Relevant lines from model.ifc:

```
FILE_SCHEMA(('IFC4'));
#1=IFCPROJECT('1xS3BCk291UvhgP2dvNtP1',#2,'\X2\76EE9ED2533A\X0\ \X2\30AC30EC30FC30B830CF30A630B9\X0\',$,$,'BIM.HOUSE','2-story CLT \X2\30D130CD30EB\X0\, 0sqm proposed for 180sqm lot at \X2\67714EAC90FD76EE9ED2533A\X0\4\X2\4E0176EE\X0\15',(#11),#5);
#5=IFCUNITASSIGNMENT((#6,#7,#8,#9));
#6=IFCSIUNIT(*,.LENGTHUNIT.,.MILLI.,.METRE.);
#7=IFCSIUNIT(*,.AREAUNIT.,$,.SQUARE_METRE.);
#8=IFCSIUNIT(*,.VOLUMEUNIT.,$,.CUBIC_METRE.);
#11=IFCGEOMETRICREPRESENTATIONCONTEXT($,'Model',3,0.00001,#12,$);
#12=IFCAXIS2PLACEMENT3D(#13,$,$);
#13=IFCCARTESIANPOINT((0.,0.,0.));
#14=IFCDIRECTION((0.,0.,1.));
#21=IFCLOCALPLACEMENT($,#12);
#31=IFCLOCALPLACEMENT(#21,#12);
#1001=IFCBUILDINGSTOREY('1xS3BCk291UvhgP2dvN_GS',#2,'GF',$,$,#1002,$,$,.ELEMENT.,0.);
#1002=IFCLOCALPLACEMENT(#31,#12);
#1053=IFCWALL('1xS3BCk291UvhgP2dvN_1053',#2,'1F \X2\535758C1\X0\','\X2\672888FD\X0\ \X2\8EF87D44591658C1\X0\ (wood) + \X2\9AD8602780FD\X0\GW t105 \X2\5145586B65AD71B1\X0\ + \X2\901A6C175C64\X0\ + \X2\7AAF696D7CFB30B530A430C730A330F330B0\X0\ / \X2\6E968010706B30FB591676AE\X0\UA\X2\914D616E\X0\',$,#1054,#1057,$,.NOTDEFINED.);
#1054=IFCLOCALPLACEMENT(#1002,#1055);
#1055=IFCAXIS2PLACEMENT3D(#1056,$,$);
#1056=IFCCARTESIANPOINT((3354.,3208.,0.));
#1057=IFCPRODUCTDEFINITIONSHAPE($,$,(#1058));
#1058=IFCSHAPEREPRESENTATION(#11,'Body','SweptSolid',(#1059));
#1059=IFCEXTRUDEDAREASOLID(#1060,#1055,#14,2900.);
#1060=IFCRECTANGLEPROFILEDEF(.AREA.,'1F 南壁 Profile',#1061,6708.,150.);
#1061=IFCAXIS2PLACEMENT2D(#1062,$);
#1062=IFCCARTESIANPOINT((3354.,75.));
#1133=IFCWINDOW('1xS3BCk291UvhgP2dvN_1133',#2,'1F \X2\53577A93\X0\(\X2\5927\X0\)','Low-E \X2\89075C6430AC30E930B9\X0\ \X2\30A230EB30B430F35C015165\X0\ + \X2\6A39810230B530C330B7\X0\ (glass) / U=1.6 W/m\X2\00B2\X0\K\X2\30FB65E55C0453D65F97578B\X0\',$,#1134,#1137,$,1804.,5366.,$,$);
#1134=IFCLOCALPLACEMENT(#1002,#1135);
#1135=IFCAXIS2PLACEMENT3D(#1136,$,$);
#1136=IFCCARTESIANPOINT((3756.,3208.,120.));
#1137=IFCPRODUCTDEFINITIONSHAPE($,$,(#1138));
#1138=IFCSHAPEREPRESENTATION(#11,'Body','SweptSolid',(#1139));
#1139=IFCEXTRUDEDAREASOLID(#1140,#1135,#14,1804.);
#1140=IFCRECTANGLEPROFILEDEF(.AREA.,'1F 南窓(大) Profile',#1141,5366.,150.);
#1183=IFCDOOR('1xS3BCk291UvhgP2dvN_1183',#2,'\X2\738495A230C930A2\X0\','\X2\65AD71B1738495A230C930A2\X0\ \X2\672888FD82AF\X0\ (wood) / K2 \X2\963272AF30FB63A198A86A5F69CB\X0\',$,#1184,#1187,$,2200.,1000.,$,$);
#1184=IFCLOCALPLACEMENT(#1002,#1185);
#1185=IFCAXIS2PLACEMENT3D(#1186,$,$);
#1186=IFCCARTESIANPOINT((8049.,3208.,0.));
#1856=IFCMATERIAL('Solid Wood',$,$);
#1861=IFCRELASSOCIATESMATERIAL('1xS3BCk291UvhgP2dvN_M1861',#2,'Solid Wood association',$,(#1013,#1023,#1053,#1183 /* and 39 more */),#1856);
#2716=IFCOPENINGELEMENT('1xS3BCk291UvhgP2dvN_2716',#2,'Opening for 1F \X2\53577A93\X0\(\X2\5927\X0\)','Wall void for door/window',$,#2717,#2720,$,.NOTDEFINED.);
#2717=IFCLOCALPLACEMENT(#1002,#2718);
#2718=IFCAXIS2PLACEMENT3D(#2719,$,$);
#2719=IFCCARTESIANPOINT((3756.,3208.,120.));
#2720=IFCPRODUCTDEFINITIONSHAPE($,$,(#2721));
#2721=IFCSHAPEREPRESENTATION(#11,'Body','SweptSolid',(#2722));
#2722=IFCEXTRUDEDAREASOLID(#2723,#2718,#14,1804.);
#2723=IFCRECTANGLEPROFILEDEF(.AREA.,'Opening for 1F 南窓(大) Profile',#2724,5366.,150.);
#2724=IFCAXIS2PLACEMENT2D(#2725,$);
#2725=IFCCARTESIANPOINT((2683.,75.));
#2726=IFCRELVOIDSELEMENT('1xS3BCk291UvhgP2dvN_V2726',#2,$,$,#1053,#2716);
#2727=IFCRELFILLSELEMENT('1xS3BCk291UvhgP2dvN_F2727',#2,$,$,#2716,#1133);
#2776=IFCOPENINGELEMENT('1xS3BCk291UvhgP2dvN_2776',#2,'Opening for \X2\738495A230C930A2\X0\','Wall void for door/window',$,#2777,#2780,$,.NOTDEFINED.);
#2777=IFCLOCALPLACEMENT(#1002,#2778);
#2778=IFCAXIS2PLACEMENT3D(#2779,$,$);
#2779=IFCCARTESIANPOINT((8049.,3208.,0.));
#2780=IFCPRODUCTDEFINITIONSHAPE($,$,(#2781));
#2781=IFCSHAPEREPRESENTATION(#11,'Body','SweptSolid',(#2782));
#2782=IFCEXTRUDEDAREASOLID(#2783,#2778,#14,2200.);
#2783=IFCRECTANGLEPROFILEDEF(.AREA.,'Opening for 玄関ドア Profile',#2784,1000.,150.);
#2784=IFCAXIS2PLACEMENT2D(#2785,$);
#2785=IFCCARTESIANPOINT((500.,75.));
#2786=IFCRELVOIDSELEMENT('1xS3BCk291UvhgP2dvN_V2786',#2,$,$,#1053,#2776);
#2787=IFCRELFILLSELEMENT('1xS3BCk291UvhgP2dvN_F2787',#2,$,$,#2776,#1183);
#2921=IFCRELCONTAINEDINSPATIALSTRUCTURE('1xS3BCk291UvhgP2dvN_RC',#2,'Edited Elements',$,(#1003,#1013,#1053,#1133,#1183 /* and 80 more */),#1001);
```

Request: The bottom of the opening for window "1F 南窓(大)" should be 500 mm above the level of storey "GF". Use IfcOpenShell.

```python
import numpy as np
import ifcopenshell
import ifcopenshell.api.geometry
import ifcopenshell.geom
import ifcopenshell.util.element
import ifcopenshell.util.placement
import ifcopenshell.util.shape
import ifcopenshell.util.unit

model = ifcopenshell.open("model.ifc")
unit_scale = ifcopenshell.util.unit.calculate_unit_scale(model)

window = model.by_guid("1xS3BCk291UvhgP2dvN_1133")
opening = window.FillsVoids[0].RelatingOpeningElement
storey = ifcopenshell.util.element.get_container(window, ifc_class="IfcBuildingStorey")
level = ifcopenshell.util.placement.get_local_placement(storey.ObjectPlacement)[2, 3]

# The opening's origin need not be at the sill, so measure its lowest point.
shape = ifcopenshell.geom.create_shape(ifcopenshell.geom.settings(), opening)
bottom = ifcopenshell.util.shape.get_shape_bottom_elevation(shape, shape.geometry) / unit_scale
dz = level + 0.5 / unit_scale - bottom

shift = np.array([0.0, 0.0, dz])
# The window is not placed relative to its opening, so move both.
for product in (opening, window):
    matrix = ifcopenshell.util.placement.get_local_placement(product.ObjectPlacement)
    matrix[:3, 3] += shift
    ifcopenshell.api.geometry.edit_object_placement(model, product=product, matrix=matrix, is_si=False)

print(f"moved by {dz * unit_scale:+.3f} m")

model.write("model_updated.ifc")
```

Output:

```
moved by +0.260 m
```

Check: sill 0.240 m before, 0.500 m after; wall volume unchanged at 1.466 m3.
